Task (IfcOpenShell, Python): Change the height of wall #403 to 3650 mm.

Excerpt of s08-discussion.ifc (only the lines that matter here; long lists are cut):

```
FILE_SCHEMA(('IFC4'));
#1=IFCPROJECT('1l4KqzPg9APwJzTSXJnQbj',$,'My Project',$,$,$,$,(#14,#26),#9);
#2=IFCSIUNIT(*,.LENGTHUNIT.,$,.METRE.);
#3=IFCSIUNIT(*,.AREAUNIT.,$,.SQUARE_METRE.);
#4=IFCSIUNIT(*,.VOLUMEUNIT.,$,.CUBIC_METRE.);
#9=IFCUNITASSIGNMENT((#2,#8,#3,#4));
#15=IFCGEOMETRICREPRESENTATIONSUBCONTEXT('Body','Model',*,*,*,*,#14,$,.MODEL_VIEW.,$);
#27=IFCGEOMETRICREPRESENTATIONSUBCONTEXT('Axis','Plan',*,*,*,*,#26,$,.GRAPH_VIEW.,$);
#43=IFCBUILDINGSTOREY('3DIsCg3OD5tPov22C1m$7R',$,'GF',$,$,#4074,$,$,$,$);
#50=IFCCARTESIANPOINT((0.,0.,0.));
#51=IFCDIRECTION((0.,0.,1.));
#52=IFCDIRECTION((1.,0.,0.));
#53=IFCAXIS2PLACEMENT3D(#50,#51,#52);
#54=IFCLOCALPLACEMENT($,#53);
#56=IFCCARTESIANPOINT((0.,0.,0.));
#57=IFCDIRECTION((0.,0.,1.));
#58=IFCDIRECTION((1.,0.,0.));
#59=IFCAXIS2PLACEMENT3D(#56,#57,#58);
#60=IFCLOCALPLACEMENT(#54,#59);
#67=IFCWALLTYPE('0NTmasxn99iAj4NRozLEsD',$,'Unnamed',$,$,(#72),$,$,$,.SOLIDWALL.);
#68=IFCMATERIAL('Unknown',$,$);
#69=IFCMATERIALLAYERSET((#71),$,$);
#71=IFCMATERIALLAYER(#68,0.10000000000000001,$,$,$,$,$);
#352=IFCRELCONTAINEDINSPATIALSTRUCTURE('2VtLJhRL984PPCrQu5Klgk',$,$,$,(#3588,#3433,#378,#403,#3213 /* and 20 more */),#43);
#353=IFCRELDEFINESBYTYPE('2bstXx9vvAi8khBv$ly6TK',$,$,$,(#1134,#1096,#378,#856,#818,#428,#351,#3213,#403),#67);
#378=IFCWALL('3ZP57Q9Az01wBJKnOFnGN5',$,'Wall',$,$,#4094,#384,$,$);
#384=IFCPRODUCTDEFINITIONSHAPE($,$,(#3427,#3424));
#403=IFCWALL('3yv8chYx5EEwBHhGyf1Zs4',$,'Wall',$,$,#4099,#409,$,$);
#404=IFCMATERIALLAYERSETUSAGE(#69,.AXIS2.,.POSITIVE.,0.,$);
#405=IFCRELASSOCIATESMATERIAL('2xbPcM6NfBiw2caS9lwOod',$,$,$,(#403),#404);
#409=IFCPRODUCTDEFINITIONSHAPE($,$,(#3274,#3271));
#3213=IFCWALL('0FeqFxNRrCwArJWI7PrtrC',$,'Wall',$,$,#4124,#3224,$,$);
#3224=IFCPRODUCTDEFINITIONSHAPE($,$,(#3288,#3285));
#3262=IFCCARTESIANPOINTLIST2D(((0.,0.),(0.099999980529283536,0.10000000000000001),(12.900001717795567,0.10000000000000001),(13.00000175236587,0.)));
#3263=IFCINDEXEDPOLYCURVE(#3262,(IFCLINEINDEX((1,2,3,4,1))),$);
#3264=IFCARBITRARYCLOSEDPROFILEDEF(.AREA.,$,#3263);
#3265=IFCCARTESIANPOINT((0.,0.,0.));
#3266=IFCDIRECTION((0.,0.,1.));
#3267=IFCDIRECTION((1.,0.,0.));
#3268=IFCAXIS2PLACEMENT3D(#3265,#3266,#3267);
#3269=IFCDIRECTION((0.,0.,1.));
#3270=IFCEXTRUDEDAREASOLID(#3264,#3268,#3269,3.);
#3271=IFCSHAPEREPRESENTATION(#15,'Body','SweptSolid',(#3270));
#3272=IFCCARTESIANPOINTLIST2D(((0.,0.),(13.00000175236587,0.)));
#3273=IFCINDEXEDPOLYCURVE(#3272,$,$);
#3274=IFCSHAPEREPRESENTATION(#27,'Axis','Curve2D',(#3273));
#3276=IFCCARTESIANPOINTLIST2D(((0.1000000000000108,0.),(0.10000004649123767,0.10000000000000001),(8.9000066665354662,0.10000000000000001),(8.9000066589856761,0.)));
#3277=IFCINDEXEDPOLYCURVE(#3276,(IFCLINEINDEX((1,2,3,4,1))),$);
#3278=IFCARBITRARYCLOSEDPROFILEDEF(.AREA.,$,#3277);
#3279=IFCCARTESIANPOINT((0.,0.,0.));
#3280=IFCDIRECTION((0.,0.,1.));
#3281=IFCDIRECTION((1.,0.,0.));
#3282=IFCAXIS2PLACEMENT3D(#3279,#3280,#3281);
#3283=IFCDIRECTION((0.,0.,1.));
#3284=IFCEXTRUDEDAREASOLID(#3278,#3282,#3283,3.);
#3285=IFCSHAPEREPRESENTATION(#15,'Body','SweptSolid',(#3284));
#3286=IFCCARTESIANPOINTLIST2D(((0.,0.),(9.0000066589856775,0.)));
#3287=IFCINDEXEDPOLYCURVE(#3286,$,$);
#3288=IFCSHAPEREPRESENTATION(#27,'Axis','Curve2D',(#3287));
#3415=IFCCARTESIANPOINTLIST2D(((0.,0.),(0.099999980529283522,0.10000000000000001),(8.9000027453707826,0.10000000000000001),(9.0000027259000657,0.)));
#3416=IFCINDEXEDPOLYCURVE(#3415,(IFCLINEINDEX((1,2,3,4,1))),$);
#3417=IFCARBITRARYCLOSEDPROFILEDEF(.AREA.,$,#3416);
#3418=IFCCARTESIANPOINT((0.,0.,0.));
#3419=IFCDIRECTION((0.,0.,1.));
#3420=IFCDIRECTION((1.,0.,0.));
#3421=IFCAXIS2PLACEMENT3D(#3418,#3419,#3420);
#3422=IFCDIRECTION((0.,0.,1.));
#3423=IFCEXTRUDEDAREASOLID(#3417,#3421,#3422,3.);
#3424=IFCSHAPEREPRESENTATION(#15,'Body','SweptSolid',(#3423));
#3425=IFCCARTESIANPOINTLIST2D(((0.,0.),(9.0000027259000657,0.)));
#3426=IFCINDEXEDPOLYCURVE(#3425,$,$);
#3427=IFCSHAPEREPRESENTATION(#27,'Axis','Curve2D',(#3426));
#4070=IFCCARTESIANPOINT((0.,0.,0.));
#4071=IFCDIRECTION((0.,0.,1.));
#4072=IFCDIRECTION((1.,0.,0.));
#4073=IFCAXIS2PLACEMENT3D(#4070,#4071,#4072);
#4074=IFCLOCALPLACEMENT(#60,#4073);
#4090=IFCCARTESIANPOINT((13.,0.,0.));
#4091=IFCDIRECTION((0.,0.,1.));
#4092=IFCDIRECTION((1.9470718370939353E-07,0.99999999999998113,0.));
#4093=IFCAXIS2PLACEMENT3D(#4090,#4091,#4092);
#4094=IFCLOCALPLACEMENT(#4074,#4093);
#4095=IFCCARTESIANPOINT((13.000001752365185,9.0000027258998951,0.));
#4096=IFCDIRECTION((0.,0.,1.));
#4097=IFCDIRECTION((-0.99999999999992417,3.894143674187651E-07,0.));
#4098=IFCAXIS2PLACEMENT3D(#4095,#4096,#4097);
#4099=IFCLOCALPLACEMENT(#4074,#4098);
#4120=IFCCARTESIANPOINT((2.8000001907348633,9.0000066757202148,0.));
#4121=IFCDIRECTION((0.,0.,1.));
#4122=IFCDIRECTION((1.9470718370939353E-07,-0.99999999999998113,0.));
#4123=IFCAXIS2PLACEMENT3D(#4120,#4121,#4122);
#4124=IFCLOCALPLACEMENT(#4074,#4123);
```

```python
import ifcopenshell
import ifcopenshell.geom
import ifcopenshell.util.representation
import ifcopenshell.util.shape
import ifcopenshell.util.unit

model = ifcopenshell.open("s08-discussion.ifc")
unit_scale = ifcopenshell.util.unit.calculate_unit_scale(model)
settings = ifcopenshell.geom.settings()


def volume(element):
    """Net volume in cubic metres, openings subtracted."""
    shape = ifcopenshell.geom.create_shape(settings, element)
    return ifcopenshell.util.shape.get_volume(shape.geometry)


wall = model.by_guid("3yv8chYx5EEwBHhGyf1Zs4")
before = volume(wall)

body = ifcopenshell.util.representation.get_representation(wall, "Model", "Body")
solid = body.Items[0]
old_height = solid.Depth
solid.Depth = 3.65 / unit_scale
after = volume(wall)

print(f"height {old_height:g} -> {solid.Depth:g}, volume {before:.3f} -> {after:.3f} m3")

model.write("s08-discussion_rev.ifc")
```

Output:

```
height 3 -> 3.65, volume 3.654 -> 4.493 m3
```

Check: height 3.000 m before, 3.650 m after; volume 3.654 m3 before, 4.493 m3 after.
